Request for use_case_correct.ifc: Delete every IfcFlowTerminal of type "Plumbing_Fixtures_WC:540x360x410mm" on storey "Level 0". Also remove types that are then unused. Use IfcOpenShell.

First a look at what the model holds.

```python
import ifcopenshell
import ifcopenshell.util.element

model = ifcopenshell.open("use_case_correct.ifc")
print(model.schema)
storey = next(s for s in model.by_type("IfcBuildingStorey") if s.Name == "Level 0")
terminals = [e for e in ifcopenshell.util.element.get_decomposition(storey) if e.is_a("IfcFlowTerminal")]
seen = {}
for e in terminals:
    element_type = ifcopenshell.util.element.get_type(e)
    name = element_type.Name if element_type not in (None, e) else None
    seen[name] = seen.get(name, 0) + 1
for name, count in sorted(seen.items(), key=str):
    print(count, "x", name)
```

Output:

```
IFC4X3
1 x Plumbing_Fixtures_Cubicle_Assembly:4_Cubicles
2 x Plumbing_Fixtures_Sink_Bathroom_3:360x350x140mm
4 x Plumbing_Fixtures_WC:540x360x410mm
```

```python
import ifcopenshell
import ifcopenshell.api.root
import ifcopenshell.util.element

model = ifcopenshell.open("use_case_correct.ifc")

storey = next(s for s in model.by_type("IfcBuildingStorey") if s.Name == "Level 0")
terminals = [e for e in ifcopenshell.util.element.get_decomposition(storey) if e.is_a("IfcFlowTerminal")]
targets = [e for e in terminals if (t := ifcopenshell.util.element.get_type(e)) not in (None, e) and t.Name == "Plumbing_Fixtures_WC:540x360x410mm"]
types = {ifcopenshell.util.element.get_type(e) for e in targets} - {None, *targets}

for e in targets:
    ifcopenshell.api.root.remove_product(model, product=e)
print(len(targets), "removed")

unused = [t for t in types if not ifcopenshell.util.element.get_types(t)]
for t in unused:
    ifcopenshell.api.root.remove_product(model, product=t)
print(len(unused), "unused types removed")

model.write("use_case_correct_updated.ifc")
```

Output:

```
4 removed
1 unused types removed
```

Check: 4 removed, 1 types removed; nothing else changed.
